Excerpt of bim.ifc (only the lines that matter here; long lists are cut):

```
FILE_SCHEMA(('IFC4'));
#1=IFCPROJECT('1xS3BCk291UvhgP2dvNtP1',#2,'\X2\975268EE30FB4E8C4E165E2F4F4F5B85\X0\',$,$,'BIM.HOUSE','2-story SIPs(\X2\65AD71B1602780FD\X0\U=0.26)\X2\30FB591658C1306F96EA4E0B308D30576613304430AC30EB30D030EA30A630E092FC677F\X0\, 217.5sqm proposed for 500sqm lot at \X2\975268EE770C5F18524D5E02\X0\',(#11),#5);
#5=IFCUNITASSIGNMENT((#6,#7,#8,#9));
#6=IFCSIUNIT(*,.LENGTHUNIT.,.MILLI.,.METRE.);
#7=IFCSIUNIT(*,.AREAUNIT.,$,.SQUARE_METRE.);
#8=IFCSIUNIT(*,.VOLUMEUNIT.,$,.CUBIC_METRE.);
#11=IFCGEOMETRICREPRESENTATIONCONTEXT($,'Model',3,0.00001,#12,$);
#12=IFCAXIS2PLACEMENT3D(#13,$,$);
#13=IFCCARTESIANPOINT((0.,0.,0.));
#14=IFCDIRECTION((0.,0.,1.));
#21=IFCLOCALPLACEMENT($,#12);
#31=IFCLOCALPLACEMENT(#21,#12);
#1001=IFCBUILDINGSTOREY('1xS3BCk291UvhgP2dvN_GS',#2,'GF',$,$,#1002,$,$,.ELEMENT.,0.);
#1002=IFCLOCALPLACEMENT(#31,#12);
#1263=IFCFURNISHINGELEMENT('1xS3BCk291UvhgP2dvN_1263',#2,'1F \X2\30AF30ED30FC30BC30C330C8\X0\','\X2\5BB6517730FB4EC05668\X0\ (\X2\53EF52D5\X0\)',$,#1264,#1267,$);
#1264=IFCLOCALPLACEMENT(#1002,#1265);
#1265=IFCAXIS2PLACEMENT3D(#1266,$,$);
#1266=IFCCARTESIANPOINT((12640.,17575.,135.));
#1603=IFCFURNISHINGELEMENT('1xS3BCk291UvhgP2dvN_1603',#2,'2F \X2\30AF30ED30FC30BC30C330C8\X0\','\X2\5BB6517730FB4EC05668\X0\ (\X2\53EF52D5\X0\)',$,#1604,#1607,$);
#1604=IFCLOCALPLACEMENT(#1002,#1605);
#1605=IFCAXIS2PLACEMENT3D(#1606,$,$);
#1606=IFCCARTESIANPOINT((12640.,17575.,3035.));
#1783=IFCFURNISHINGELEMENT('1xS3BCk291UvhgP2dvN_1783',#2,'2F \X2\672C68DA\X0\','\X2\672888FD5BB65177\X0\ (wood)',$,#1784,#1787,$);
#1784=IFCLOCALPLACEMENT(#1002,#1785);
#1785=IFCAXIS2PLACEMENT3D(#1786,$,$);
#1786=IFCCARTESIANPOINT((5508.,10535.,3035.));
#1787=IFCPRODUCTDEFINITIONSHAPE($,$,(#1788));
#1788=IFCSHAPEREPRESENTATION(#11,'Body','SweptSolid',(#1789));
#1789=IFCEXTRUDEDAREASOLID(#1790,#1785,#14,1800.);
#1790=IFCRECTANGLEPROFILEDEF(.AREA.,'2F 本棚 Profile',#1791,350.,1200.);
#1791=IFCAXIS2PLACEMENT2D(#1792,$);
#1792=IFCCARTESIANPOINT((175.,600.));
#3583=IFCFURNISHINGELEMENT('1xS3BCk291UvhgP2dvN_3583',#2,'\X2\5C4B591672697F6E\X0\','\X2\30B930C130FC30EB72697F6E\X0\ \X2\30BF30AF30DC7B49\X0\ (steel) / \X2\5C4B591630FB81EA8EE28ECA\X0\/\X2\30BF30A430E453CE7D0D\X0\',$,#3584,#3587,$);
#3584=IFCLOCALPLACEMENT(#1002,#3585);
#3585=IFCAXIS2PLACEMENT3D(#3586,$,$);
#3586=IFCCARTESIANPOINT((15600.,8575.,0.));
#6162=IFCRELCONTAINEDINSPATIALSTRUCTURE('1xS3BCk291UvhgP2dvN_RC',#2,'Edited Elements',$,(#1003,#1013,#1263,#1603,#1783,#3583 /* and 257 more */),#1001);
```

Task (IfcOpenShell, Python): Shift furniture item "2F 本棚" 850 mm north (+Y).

```python
import ifcopenshell
import ifcopenshell.api.geometry
import ifcopenshell.util.placement

model = ifcopenshell.open("bim.ifc")

item = model.by_guid("1xS3BCk291UvhgP2dvN_1783")
matrix = ifcopenshell.util.placement.get_local_placement(item.ObjectPlacement)
matrix[1, 3] += 850.0
ifcopenshell.api.geometry.edit_object_placement(model, product=item, matrix=matrix, is_si=False)

print(ifcopenshell.util.placement.get_local_placement(item.ObjectPlacement).round(3) + 0.0)

model.write("bim_rev.ifc")
```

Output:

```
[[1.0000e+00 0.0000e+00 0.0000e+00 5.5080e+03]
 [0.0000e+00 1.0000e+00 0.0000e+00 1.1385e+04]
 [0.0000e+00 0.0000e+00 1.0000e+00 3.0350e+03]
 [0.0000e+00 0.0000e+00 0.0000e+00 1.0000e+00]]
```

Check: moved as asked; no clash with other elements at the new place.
